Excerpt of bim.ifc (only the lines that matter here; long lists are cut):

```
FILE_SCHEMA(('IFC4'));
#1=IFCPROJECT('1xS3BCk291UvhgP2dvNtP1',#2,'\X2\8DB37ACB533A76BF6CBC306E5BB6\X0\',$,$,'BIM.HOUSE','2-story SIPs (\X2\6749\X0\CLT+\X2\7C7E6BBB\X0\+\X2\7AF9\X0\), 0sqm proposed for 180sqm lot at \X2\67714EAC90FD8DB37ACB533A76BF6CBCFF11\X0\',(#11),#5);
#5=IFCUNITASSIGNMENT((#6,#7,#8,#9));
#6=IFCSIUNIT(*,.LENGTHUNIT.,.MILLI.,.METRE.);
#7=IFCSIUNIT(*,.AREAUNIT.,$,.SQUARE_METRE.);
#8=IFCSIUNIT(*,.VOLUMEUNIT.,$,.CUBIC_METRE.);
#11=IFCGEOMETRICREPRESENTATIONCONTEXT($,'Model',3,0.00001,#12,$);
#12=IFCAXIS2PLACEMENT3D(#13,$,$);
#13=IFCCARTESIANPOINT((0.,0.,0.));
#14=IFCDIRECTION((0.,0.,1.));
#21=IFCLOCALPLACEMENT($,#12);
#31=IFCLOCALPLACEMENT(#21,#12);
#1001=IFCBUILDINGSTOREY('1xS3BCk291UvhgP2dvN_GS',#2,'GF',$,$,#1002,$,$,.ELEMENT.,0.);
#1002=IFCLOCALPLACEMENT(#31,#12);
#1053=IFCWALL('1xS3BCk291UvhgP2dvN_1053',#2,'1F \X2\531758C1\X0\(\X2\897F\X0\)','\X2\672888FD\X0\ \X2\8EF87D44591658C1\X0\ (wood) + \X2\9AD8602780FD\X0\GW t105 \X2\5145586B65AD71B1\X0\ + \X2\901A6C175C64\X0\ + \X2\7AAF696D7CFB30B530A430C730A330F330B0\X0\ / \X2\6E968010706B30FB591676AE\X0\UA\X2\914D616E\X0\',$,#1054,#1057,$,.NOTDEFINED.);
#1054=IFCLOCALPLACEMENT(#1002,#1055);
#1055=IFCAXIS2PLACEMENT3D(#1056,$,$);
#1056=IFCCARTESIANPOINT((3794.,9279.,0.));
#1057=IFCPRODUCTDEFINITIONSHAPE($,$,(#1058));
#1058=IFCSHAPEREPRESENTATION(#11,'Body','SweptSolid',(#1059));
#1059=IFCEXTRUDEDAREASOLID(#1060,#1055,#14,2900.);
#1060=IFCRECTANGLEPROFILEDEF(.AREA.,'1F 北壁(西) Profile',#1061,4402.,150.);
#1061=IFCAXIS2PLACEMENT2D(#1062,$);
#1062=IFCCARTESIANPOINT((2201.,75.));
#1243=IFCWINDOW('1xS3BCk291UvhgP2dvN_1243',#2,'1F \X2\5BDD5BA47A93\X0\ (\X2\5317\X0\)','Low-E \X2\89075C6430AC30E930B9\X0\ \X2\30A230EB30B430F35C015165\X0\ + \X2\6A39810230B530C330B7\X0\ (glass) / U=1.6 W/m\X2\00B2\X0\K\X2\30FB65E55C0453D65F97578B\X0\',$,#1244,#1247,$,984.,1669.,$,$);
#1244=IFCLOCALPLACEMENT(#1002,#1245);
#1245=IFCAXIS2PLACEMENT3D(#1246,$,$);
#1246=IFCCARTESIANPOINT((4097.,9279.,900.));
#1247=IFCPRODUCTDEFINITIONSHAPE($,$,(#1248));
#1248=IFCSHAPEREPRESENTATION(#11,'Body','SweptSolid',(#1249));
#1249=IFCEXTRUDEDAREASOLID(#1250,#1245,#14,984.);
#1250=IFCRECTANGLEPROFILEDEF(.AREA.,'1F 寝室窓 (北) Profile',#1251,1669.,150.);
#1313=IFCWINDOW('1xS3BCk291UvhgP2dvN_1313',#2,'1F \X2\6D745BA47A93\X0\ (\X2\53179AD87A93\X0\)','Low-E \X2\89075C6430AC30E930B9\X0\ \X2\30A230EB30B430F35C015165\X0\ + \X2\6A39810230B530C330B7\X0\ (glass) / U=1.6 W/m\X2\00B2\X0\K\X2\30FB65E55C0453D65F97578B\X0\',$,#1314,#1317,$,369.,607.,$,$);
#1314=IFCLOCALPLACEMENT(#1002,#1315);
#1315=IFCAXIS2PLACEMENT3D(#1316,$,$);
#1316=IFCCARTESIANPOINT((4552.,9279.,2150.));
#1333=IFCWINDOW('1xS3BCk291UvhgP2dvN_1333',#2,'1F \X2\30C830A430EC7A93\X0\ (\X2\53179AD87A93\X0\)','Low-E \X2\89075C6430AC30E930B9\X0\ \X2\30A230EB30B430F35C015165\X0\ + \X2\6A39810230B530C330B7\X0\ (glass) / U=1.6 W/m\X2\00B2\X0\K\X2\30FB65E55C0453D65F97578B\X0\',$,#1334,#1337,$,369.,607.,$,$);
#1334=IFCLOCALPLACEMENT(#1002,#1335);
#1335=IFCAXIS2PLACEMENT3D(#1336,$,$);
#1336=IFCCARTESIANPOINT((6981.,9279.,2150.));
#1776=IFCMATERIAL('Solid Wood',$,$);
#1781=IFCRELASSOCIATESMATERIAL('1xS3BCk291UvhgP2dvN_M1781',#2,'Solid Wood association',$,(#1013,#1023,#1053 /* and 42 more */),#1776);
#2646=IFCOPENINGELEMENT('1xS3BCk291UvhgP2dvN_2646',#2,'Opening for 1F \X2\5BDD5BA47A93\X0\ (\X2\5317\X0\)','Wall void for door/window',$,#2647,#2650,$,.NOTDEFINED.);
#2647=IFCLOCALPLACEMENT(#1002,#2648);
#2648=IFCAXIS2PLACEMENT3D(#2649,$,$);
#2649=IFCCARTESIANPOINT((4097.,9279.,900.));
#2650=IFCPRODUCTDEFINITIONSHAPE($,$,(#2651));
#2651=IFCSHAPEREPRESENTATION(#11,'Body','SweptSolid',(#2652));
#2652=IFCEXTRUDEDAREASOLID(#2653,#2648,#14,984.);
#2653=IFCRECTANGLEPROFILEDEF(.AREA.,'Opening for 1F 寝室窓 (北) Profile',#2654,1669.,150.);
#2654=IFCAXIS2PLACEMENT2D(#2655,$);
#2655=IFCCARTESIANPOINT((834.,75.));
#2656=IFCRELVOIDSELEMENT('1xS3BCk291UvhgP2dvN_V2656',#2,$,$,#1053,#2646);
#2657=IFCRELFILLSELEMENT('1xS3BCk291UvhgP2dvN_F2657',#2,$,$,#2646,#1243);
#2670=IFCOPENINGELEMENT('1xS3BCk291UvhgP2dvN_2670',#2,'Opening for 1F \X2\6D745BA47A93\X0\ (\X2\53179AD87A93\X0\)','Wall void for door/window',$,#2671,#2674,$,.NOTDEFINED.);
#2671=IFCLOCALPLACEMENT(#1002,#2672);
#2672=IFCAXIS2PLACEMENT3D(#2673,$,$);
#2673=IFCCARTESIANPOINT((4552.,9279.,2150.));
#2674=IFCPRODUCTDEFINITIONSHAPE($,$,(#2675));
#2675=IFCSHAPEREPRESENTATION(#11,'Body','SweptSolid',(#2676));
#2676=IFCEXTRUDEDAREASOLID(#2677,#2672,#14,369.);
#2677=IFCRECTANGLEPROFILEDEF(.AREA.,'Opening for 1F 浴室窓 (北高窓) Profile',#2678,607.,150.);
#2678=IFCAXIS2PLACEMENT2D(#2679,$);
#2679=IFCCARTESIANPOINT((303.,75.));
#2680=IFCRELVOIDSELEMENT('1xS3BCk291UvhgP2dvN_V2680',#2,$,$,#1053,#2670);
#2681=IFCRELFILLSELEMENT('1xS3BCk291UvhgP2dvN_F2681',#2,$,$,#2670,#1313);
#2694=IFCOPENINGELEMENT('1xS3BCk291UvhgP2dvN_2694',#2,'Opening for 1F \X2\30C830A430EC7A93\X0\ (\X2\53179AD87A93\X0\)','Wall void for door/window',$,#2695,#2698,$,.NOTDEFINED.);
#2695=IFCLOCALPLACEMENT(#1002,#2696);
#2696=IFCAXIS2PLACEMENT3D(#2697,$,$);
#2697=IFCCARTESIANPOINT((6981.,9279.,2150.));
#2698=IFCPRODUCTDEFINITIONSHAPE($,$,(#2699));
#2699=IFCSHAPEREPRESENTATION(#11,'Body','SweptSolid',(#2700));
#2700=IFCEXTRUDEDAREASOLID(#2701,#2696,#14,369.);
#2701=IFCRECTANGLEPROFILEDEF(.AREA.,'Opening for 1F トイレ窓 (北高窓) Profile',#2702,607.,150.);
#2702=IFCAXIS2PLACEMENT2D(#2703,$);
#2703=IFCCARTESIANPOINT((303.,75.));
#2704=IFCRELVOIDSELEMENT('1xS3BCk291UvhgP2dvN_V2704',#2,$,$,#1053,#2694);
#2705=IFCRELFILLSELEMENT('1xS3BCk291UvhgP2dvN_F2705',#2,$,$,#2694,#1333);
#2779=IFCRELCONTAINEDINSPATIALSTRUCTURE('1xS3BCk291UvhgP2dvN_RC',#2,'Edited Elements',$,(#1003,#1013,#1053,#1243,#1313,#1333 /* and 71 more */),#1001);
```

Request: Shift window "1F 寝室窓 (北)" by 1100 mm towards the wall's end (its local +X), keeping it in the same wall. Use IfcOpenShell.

```python
import ifcopenshell
import ifcopenshell.api.geometry
import ifcopenshell.util.placement

model = ifcopenshell.open("bim.ifc")

window = model.by_guid("1xS3BCk291UvhgP2dvN_1243")
opening = window.FillsVoids[0].RelatingOpeningElement
wall = opening.VoidsElements[0].RelatingBuildingElement

wall_matrix = ifcopenshell.util.placement.get_local_placement(wall.ObjectPlacement)
shift = wall_matrix[:3, 0] * 1100.0
before = ifcopenshell.util.placement.get_local_placement(window.ObjectPlacement)[:3, 3].copy()

# The window is not placed relative to its opening, so move both.
for product in (opening, window):
    matrix = ifcopenshell.util.placement.get_local_placement(product.ObjectPlacement)
    matrix[:3, 3] += shift
    ifcopenshell.api.geometry.edit_object_placement(model, product=product, matrix=matrix, is_si=False)

after = ifcopenshell.util.placement.get_local_placement(window.ObjectPlacement)[:3, 3]
print("window moved by", (after - before).round(3) + 0.0)

model.write("bim_edited.ifc")
```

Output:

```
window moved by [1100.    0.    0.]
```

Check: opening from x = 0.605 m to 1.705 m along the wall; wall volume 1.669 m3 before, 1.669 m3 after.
